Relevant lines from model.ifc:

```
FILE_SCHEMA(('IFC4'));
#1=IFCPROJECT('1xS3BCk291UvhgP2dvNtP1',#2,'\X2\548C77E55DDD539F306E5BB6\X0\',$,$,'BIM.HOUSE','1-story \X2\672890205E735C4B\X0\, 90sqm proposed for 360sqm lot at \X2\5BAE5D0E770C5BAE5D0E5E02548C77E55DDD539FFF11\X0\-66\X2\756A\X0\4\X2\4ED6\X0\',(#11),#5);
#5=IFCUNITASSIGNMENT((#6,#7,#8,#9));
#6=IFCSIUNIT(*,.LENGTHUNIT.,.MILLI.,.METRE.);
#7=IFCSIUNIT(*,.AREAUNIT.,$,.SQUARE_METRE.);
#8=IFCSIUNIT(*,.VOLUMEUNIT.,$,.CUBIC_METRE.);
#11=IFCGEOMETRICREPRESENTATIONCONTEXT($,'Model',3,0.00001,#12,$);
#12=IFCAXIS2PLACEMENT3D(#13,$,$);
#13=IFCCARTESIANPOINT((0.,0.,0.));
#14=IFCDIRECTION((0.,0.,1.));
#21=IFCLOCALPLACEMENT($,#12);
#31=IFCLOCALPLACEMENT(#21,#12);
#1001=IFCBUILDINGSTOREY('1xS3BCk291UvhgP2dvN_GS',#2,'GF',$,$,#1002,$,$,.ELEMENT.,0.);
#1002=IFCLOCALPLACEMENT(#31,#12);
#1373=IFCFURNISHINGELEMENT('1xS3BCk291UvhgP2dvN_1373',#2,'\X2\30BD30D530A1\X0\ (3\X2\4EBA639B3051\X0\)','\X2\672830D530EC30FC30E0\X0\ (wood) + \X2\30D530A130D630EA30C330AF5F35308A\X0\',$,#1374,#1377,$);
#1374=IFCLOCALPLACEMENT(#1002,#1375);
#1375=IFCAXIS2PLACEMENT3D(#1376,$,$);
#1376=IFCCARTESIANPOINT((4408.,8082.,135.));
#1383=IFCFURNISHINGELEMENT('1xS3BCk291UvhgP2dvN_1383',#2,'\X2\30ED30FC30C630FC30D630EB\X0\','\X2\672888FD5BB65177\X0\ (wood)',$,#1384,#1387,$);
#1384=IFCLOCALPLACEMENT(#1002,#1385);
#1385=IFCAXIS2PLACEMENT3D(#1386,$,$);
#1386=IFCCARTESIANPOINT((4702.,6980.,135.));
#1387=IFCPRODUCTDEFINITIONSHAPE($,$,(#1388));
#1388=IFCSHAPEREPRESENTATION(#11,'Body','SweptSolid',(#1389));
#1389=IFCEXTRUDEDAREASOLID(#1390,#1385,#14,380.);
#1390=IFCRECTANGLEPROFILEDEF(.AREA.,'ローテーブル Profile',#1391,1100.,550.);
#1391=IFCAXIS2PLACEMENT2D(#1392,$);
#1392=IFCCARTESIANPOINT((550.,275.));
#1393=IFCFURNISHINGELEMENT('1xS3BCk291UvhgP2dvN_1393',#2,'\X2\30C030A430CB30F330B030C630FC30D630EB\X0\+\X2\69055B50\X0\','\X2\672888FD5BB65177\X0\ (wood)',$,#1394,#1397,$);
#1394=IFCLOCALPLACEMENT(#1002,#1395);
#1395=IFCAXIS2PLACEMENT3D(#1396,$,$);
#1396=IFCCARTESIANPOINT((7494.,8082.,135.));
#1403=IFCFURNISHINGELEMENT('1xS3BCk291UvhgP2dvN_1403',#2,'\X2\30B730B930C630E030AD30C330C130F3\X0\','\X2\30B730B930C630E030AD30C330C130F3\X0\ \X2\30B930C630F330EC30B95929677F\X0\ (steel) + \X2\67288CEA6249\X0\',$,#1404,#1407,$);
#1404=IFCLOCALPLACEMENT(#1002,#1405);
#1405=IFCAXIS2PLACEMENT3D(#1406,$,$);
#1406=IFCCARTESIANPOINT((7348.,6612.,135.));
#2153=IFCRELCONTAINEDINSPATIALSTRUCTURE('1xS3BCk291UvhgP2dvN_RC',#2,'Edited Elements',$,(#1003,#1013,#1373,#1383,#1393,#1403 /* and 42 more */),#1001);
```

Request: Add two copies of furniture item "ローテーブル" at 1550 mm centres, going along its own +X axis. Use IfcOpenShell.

```python
import ifcopenshell
import ifcopenshell.api.geometry
import ifcopenshell.api.root
import ifcopenshell.util.element
import ifcopenshell.util.placement

model = ifcopenshell.open("model.ifc")


def reuse_history(source, copy):
    """copy_class also copies each property set's owner history, people and application; keep the originals."""
    for rel in copy.IsDefinedBy:
        if rel.is_a("IfcRelDefinesByProperties") and (history := rel.RelatingPropertyDefinition.OwnerHistory):
            rel.RelatingPropertyDefinition.OwnerHistory = source.OwnerHistory
            ifcopenshell.util.element.remove_deep2(model, history)


source = model.by_guid("1xS3BCk291UvhgP2dvN_1383")
base = ifcopenshell.util.placement.get_local_placement(source.ObjectPlacement)
step = base[:3, 0] * 1550.0

for i in range(1, 3):
    copy = ifcopenshell.api.root.copy_class(model, product=source)
    copy.Representation = ifcopenshell.util.element.copy_deep(
        model, source.Representation, exclude=["IfcGeometricRepresentationContext", "IfcRepresentationMap"]
    )
    reuse_history(source, copy)
    matrix = base.copy()
    matrix[:3, 3] += i * step
    print("added at", matrix[:3, 3].round(3) + 0.0)
    ifcopenshell.api.geometry.edit_object_placement(model, product=copy, matrix=matrix, is_si=False)

model.write("model-out.ifc")
```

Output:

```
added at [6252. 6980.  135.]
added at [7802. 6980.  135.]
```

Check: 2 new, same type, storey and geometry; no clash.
